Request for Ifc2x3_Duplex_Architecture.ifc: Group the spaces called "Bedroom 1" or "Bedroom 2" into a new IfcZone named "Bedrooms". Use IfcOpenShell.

First a look at what the model holds.

```python
import ifcopenshell

model = ifcopenshell.open("Ifc2x3_Duplex_Architecture.ifc")
print(model.schema)
seen = {}
for space in model.by_type("IfcSpace"):
    seen[space.LongName] = seen.get(space.LongName, 0) + 1
for name, count in sorted(seen.items(), key=str):
    print(count, "x", name)
print("zones:", [z.Name for z in model.by_type("IfcZone")][:20])
```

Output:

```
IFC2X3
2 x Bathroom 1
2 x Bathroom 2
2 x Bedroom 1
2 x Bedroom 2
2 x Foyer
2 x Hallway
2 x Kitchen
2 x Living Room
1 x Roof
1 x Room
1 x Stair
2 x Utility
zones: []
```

```python
import ifcopenshell
import ifcopenshell.api.group
import ifcopenshell.api.root

model = ifcopenshell.open("Ifc2x3_Duplex_Architecture.ifc")

names = {"Bedroom 1", "Bedroom 2"}
spaces = [s for s in model.by_type("IfcSpace") if s.LongName in names]

zone = ifcopenshell.api.root.create_entity(model, ifc_class="IfcZone", name="Bedrooms")
ifcopenshell.api.group.assign_group(model, products=spaces, group=zone)
print(len(spaces), "spaces in", zone.Name)

model.write("Ifc2x3_Duplex_Architecture_edited.ifc")
```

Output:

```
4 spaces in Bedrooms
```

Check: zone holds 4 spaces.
